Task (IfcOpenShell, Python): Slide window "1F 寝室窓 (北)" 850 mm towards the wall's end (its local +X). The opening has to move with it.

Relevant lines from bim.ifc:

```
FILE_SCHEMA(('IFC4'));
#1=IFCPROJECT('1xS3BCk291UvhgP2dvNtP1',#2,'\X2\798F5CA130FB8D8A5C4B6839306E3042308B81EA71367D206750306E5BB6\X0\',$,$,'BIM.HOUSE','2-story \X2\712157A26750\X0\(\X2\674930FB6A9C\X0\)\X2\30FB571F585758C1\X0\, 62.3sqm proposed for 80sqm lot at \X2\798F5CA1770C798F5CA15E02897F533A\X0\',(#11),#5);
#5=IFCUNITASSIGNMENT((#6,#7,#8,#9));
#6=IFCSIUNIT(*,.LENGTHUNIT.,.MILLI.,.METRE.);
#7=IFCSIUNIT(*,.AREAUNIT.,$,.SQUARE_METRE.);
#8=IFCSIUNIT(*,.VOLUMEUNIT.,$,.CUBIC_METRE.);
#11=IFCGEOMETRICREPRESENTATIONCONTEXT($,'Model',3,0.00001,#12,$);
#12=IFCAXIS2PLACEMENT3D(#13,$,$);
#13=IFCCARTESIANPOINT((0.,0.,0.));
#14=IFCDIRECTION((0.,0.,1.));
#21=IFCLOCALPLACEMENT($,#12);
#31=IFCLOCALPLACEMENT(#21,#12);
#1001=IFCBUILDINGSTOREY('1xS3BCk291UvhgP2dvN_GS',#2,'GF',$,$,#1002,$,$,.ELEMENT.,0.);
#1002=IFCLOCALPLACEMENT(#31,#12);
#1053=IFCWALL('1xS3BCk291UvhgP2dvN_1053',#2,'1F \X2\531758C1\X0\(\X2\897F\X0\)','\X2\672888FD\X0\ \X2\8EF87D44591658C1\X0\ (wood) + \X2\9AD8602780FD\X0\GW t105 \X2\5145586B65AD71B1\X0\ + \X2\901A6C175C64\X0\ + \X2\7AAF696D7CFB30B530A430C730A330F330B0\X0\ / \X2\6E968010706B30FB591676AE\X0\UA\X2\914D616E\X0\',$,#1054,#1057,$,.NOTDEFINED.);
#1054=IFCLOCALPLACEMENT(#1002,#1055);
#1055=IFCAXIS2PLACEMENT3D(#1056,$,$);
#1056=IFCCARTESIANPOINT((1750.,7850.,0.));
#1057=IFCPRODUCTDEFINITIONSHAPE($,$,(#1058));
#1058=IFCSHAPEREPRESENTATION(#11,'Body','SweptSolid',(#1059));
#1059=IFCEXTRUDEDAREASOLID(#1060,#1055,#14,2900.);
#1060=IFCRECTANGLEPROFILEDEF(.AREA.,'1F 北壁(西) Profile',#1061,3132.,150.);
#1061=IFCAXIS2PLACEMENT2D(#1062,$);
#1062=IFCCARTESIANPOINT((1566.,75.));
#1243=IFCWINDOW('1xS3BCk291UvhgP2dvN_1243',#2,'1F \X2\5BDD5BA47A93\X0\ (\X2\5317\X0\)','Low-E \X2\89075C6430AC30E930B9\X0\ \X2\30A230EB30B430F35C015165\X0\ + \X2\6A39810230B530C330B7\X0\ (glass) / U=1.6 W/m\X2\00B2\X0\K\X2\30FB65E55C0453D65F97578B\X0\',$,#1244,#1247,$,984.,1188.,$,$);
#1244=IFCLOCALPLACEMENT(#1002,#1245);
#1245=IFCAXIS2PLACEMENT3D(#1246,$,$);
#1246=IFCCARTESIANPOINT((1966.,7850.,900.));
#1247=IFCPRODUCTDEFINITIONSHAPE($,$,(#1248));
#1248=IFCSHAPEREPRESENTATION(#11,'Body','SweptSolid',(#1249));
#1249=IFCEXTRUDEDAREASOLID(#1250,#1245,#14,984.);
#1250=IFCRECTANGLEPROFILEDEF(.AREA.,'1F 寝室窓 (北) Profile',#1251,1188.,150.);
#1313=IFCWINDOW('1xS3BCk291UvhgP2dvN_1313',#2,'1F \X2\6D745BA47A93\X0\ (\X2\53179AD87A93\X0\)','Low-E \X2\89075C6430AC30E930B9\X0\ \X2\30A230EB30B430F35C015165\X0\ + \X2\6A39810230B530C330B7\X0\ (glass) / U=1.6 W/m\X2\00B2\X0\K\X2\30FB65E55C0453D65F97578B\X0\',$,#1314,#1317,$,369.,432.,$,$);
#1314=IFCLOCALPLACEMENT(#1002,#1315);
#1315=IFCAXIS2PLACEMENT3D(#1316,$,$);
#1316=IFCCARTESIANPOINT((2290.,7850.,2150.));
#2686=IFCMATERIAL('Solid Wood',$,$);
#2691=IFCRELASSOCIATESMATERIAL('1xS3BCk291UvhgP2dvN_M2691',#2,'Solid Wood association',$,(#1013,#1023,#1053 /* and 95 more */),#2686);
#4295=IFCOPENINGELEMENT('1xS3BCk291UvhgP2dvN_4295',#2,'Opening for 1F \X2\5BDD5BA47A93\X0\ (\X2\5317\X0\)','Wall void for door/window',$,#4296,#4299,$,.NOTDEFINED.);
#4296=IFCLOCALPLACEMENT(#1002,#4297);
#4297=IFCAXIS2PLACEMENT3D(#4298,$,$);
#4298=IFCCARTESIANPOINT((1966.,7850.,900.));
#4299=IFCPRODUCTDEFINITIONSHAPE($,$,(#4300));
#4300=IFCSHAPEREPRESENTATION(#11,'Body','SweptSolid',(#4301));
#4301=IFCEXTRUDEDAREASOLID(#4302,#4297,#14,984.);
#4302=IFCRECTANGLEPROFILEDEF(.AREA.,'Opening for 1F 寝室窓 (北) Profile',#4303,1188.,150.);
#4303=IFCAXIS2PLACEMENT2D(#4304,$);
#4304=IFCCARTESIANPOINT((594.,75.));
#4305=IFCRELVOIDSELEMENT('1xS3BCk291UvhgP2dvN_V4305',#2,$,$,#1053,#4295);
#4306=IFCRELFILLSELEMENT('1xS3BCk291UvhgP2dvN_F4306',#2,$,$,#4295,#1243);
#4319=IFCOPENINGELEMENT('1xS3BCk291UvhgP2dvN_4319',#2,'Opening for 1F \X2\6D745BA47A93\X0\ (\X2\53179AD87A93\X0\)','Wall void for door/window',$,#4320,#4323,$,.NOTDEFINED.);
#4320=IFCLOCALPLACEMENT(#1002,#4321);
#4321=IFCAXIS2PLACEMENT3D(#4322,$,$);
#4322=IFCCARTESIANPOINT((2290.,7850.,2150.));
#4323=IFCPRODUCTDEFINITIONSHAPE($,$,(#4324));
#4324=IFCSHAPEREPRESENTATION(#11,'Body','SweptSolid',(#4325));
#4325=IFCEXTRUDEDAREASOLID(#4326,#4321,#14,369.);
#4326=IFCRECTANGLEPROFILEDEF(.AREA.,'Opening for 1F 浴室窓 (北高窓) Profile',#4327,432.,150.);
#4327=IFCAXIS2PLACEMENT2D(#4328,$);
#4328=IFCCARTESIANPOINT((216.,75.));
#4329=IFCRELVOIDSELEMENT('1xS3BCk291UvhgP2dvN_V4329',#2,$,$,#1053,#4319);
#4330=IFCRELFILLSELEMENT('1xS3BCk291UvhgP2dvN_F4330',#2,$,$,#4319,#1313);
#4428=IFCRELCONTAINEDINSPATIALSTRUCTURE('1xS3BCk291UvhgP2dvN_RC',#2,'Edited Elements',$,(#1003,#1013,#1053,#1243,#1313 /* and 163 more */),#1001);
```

```python
import ifcopenshell
import ifcopenshell.api.geometry
import ifcopenshell.util.placement

model = ifcopenshell.open("bim.ifc")

window = model.by_guid("1xS3BCk291UvhgP2dvN_1243")
opening = window.FillsVoids[0].RelatingOpeningElement
wall = opening.VoidsElements[0].RelatingBuildingElement

wall_matrix = ifcopenshell.util.placement.get_local_placement(wall.ObjectPlacement)
shift = wall_matrix[:3, 0] * 850.0
before = ifcopenshell.util.placement.get_local_placement(window.ObjectPlacement)[:3, 3].copy()

# The window is not placed relative to its opening, so move both.
for product in (opening, window):
    matrix = ifcopenshell.util.placement.get_local_placement(product.ObjectPlacement)
    matrix[:3, 3] += shift
    ifcopenshell.api.geometry.edit_object_placement(model, product=product, matrix=matrix, is_si=False)

after = ifcopenshell.util.placement.get_local_placement(window.ObjectPlacement)[:3, 3]
print("window moved by", (after - before).round(3) + 0.0)

model.write("bim-out.ifc")
```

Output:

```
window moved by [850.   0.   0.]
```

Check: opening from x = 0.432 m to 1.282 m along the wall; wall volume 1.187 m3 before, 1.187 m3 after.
